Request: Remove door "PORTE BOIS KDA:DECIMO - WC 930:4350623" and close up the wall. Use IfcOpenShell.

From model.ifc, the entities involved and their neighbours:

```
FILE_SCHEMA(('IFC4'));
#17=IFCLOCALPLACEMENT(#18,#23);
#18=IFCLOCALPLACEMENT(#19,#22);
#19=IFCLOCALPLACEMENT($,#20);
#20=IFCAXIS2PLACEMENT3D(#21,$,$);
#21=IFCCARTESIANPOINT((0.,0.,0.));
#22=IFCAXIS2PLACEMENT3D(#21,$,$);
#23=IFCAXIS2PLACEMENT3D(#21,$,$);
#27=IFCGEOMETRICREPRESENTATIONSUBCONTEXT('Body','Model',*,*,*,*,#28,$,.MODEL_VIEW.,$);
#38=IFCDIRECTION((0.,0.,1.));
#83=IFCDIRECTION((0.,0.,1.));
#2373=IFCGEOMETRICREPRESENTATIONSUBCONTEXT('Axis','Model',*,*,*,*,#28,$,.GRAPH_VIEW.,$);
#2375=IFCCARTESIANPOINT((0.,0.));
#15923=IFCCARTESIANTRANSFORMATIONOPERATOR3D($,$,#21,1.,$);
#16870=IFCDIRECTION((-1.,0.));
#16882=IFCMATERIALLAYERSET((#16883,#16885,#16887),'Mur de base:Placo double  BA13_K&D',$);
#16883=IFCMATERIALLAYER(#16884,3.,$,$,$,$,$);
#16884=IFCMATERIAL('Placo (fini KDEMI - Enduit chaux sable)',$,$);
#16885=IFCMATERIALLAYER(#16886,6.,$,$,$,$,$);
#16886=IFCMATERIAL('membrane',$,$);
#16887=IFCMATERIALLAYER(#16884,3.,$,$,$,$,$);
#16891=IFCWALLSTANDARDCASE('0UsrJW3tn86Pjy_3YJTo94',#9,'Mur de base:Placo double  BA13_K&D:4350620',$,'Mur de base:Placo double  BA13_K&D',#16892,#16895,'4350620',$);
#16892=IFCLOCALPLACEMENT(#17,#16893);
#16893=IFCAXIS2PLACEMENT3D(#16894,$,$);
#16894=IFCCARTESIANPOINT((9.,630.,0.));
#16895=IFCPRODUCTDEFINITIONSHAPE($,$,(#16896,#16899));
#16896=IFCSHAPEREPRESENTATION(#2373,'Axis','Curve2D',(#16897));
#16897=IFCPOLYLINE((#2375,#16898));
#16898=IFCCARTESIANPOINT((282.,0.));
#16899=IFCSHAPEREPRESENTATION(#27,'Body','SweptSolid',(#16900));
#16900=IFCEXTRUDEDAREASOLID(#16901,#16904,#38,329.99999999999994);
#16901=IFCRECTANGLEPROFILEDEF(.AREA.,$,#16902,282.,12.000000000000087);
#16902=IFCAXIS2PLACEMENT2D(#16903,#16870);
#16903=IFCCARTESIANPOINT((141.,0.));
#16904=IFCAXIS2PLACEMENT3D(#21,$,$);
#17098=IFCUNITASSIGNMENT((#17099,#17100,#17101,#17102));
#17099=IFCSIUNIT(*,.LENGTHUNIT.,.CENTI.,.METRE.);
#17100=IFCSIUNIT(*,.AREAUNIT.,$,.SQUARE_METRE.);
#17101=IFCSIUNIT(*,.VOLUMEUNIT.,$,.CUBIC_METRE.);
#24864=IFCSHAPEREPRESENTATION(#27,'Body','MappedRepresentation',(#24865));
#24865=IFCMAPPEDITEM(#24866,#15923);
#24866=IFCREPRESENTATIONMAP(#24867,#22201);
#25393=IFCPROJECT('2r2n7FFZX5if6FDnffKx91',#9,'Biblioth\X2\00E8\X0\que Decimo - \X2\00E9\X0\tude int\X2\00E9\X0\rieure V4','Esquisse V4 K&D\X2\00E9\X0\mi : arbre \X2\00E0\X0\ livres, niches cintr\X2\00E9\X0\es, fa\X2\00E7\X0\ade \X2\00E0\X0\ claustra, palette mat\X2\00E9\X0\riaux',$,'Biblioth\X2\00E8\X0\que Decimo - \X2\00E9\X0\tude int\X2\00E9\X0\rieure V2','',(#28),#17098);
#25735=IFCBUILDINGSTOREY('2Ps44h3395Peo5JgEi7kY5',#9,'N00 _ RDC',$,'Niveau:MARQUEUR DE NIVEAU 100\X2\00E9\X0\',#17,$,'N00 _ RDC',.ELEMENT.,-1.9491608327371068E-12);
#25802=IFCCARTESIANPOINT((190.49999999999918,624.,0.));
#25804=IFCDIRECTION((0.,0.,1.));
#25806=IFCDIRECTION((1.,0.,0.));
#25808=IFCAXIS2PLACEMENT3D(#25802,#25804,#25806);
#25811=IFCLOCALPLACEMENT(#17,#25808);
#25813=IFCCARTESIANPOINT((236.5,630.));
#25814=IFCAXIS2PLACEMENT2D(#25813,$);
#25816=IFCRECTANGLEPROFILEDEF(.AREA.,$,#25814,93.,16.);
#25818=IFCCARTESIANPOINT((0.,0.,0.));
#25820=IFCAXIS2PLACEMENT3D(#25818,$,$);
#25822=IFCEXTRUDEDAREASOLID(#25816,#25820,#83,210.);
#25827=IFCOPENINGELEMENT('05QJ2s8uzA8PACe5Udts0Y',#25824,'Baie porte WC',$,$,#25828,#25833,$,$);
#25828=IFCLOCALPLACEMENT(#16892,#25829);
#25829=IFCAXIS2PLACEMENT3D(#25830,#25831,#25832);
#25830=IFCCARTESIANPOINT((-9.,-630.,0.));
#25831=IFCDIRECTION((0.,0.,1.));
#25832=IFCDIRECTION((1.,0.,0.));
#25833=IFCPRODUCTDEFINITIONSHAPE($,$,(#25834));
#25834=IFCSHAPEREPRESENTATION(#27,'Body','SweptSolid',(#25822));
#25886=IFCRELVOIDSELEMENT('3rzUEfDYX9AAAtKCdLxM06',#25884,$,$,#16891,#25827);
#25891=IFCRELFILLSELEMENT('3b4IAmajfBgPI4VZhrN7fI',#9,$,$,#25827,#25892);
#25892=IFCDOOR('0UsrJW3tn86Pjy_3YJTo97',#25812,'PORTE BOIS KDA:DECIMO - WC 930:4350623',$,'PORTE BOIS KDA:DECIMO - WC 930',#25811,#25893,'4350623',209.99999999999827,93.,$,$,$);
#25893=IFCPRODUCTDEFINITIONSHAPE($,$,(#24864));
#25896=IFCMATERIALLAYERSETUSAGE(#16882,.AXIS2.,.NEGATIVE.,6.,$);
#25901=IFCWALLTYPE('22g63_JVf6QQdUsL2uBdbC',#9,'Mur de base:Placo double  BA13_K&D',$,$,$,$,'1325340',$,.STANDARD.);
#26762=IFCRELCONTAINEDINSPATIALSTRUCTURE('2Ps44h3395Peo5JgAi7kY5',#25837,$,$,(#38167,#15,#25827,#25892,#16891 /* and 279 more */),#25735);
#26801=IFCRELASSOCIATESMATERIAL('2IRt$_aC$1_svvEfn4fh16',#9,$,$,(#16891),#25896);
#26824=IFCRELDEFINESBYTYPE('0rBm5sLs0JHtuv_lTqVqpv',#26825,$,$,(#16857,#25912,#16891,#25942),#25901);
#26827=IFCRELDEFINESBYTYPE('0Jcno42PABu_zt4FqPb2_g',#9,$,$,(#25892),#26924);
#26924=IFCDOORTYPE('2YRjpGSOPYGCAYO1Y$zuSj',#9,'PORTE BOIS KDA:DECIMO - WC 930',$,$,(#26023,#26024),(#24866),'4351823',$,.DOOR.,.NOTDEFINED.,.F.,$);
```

```python
import ifcopenshell
import ifcopenshell.api.feature
import ifcopenshell.api.root
import ifcopenshell.geom
import ifcopenshell.util.shape

model = ifcopenshell.open("model.ifc")
settings = ifcopenshell.geom.settings()


def volume(element):
    """Net volume in cubic metres, openings subtracted."""
    shape = ifcopenshell.geom.create_shape(settings, element)
    return ifcopenshell.util.shape.get_volume(shape.geometry)


door = model.by_guid("0UsrJW3tn86Pjy_3YJTo97")
opening = door.FillsVoids[0].RelatingOpeningElement
wall = opening.VoidsElements[0].RelatingBuildingElement
before = volume(wall)

ifcopenshell.api.root.remove_product(model, product=door)
ifcopenshell.api.feature.remove_feature(model, feature=opening)

after = volume(wall)

print(f"wall volume {before:.3f} -> {after:.3f} m3")

model.write("model-out.ifc")
```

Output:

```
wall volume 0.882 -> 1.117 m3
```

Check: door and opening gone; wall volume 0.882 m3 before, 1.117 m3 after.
